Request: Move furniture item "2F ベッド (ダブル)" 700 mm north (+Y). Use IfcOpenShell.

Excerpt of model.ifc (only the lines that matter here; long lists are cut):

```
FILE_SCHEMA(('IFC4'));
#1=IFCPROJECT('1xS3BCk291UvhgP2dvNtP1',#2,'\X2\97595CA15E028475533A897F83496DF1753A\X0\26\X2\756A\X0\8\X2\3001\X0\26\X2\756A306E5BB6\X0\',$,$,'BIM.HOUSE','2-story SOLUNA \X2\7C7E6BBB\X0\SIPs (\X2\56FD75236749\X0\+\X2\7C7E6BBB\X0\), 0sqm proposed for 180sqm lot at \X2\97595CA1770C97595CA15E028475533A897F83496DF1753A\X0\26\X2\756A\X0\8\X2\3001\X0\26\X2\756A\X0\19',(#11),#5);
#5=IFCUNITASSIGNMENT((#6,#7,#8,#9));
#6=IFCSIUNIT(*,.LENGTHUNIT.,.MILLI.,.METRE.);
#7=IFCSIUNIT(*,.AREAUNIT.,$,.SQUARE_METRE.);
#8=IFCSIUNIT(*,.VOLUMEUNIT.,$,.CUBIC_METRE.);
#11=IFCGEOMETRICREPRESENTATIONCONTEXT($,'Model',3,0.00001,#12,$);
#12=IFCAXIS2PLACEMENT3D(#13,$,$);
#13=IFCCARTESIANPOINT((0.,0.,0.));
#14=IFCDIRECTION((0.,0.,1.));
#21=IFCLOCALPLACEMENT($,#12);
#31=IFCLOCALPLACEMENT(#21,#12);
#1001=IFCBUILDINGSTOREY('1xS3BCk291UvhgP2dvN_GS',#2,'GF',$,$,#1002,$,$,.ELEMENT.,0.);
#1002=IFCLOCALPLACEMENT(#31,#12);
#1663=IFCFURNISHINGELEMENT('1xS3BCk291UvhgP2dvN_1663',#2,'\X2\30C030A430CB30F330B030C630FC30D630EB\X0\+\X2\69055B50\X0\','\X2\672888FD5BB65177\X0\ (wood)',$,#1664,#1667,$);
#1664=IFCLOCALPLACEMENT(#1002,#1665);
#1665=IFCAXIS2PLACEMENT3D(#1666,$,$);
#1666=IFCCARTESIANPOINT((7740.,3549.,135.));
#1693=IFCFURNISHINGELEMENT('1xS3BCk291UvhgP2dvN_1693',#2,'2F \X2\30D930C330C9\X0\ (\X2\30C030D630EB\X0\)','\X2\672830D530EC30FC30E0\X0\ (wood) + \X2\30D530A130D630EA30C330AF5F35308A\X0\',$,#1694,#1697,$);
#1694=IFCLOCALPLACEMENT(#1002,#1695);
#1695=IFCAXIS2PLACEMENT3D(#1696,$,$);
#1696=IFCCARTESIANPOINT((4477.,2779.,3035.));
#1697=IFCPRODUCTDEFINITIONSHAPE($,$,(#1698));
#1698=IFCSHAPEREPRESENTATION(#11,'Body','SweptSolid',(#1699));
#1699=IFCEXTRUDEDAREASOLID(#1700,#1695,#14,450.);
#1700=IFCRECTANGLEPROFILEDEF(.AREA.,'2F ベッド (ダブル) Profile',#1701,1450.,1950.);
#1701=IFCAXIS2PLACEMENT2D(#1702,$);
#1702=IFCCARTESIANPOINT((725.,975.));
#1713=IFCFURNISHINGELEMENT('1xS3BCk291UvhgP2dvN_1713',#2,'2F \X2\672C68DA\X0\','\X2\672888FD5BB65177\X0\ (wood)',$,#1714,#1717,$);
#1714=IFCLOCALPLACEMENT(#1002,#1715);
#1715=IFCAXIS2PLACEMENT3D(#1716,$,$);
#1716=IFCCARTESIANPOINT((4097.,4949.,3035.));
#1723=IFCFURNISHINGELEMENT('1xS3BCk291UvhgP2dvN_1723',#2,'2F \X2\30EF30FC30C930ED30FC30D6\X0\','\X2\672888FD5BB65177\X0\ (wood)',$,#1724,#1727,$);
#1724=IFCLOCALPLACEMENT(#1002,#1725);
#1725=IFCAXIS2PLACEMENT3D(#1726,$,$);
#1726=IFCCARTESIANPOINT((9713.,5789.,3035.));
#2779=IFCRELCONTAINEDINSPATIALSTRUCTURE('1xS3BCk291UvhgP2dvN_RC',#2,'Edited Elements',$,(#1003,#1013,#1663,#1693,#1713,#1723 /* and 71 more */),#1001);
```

```python
import ifcopenshell
import ifcopenshell.api.geometry
import ifcopenshell.util.placement

model = ifcopenshell.open("model.ifc")

item = model.by_id(1693)
matrix = ifcopenshell.util.placement.get_local_placement(item.ObjectPlacement)
matrix[1, 3] += 700.0
ifcopenshell.api.geometry.edit_object_placement(model, product=item, matrix=matrix, is_si=False)

print(ifcopenshell.util.placement.get_local_placement(item.ObjectPlacement).round(3) + 0.0)

model.write("model_edited.ifc")
```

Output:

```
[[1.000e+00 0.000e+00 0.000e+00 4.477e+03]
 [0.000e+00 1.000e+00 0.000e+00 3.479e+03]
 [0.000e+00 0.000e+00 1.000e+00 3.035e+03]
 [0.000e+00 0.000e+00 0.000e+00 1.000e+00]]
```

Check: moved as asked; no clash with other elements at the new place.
